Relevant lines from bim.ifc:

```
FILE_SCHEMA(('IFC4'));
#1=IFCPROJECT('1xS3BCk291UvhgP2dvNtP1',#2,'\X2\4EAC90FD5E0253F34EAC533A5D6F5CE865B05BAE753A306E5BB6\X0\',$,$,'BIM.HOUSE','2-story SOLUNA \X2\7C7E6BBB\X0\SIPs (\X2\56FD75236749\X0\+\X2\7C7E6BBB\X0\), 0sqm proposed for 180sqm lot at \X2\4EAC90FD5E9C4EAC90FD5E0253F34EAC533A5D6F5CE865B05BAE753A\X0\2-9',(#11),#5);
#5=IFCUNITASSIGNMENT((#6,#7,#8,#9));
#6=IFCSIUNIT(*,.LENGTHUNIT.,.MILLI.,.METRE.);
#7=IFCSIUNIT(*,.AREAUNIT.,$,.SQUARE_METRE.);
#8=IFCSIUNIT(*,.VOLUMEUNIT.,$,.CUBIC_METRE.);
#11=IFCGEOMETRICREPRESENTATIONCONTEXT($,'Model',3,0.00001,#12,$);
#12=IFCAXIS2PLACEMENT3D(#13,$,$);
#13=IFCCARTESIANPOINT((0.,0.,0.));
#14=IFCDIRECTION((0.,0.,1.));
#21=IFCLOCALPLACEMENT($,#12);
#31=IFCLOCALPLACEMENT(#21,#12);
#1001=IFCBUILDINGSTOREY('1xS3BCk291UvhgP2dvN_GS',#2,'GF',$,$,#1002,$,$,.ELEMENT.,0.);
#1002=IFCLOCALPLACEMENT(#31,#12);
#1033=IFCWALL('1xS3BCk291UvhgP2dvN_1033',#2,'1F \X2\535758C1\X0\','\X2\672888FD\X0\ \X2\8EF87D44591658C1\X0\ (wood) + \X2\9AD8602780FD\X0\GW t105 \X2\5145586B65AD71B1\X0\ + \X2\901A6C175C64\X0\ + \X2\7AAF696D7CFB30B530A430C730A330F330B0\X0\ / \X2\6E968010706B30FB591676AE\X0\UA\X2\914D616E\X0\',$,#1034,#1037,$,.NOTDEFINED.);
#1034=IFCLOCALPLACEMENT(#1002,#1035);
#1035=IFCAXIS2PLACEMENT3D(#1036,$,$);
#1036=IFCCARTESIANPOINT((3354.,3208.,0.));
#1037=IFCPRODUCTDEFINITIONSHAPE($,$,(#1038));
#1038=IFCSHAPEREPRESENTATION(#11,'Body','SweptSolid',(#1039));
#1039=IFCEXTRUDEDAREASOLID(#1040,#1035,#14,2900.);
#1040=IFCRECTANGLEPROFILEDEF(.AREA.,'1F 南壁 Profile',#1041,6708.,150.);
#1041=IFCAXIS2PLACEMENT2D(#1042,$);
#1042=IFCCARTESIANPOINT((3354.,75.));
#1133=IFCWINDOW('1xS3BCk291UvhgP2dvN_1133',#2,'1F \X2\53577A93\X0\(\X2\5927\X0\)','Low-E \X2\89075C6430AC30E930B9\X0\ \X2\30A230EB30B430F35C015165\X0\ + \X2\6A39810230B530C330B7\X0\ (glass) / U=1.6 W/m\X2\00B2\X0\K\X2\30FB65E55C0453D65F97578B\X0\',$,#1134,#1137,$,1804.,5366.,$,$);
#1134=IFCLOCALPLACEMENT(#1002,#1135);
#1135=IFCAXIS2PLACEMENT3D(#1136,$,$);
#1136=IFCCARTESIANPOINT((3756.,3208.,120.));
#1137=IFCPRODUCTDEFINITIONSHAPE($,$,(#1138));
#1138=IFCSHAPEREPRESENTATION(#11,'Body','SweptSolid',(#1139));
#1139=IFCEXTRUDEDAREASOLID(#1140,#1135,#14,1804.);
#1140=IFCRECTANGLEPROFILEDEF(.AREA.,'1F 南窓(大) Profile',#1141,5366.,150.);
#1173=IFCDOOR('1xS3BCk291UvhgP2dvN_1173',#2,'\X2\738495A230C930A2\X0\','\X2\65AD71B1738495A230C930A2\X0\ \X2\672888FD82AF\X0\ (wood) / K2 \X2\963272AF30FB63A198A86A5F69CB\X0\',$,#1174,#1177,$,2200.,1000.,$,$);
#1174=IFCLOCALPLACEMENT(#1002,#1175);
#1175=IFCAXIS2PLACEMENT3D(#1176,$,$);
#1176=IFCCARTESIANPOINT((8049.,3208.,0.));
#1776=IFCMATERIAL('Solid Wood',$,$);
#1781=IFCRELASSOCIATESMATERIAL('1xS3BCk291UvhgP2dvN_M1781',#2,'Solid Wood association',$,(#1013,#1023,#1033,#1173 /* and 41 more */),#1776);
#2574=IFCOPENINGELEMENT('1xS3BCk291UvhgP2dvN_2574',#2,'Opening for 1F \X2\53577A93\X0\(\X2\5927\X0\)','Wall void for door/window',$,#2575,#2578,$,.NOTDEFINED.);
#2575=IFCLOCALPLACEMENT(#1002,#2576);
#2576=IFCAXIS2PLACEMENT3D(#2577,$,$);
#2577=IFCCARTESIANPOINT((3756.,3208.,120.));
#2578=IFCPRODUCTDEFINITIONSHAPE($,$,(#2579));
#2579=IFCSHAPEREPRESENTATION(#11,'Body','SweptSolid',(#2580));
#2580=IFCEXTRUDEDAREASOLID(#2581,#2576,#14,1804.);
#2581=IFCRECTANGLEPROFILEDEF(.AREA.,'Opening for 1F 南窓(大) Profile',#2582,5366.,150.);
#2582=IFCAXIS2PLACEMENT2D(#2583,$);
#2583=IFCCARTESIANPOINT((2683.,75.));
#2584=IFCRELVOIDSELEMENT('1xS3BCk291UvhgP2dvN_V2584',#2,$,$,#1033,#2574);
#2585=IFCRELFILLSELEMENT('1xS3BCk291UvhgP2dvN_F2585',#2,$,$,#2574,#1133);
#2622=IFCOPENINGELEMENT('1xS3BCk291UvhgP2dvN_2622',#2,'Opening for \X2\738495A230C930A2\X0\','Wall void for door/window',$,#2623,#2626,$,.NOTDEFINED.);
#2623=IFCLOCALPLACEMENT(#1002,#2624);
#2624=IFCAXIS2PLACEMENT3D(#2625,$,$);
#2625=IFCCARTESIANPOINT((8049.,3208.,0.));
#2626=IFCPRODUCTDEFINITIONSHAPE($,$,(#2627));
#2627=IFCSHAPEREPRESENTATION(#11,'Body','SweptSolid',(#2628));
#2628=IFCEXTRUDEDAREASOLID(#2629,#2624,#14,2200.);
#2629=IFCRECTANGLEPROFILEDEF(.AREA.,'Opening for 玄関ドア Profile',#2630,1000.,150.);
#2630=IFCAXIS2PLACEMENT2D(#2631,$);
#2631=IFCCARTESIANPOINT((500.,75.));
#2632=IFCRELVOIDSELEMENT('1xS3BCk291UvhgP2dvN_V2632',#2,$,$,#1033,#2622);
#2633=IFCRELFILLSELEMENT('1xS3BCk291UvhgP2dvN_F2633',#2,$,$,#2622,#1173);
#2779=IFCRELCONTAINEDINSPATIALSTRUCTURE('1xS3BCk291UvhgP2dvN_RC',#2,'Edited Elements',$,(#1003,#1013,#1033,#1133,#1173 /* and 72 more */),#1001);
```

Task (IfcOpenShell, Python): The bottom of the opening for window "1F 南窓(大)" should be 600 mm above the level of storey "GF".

```python
import numpy as np
import ifcopenshell
import ifcopenshell.api.geometry
import ifcopenshell.geom
import ifcopenshell.util.element
import ifcopenshell.util.placement
import ifcopenshell.util.shape
import ifcopenshell.util.unit

model = ifcopenshell.open("bim.ifc")
unit_scale = ifcopenshell.util.unit.calculate_unit_scale(model)

window = model.by_id(1133)
opening = window.FillsVoids[0].RelatingOpeningElement
storey = ifcopenshell.util.element.get_container(window, ifc_class="IfcBuildingStorey")
level = ifcopenshell.util.placement.get_local_placement(storey.ObjectPlacement)[2, 3]

# The opening's origin need not be at the sill, so measure its lowest point.
shape = ifcopenshell.geom.create_shape(ifcopenshell.geom.settings(), opening)
bottom = ifcopenshell.util.shape.get_shape_bottom_elevation(shape, shape.geometry) / unit_scale
dz = level + 600.0 - bottom

shift = np.array([0.0, 0.0, dz])
# The window is not placed relative to its opening, so move both.
for product in (opening, window):
    matrix = ifcopenshell.util.placement.get_local_placement(product.ObjectPlacement)
    matrix[:3, 3] += shift
    ifcopenshell.api.geometry.edit_object_placement(model, product=product, matrix=matrix, is_si=False)

print(f"moved by {dz * unit_scale:+.3f} m")

model.write("bim_rev.ifc")
```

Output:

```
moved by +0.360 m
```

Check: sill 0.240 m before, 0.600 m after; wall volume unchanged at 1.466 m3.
